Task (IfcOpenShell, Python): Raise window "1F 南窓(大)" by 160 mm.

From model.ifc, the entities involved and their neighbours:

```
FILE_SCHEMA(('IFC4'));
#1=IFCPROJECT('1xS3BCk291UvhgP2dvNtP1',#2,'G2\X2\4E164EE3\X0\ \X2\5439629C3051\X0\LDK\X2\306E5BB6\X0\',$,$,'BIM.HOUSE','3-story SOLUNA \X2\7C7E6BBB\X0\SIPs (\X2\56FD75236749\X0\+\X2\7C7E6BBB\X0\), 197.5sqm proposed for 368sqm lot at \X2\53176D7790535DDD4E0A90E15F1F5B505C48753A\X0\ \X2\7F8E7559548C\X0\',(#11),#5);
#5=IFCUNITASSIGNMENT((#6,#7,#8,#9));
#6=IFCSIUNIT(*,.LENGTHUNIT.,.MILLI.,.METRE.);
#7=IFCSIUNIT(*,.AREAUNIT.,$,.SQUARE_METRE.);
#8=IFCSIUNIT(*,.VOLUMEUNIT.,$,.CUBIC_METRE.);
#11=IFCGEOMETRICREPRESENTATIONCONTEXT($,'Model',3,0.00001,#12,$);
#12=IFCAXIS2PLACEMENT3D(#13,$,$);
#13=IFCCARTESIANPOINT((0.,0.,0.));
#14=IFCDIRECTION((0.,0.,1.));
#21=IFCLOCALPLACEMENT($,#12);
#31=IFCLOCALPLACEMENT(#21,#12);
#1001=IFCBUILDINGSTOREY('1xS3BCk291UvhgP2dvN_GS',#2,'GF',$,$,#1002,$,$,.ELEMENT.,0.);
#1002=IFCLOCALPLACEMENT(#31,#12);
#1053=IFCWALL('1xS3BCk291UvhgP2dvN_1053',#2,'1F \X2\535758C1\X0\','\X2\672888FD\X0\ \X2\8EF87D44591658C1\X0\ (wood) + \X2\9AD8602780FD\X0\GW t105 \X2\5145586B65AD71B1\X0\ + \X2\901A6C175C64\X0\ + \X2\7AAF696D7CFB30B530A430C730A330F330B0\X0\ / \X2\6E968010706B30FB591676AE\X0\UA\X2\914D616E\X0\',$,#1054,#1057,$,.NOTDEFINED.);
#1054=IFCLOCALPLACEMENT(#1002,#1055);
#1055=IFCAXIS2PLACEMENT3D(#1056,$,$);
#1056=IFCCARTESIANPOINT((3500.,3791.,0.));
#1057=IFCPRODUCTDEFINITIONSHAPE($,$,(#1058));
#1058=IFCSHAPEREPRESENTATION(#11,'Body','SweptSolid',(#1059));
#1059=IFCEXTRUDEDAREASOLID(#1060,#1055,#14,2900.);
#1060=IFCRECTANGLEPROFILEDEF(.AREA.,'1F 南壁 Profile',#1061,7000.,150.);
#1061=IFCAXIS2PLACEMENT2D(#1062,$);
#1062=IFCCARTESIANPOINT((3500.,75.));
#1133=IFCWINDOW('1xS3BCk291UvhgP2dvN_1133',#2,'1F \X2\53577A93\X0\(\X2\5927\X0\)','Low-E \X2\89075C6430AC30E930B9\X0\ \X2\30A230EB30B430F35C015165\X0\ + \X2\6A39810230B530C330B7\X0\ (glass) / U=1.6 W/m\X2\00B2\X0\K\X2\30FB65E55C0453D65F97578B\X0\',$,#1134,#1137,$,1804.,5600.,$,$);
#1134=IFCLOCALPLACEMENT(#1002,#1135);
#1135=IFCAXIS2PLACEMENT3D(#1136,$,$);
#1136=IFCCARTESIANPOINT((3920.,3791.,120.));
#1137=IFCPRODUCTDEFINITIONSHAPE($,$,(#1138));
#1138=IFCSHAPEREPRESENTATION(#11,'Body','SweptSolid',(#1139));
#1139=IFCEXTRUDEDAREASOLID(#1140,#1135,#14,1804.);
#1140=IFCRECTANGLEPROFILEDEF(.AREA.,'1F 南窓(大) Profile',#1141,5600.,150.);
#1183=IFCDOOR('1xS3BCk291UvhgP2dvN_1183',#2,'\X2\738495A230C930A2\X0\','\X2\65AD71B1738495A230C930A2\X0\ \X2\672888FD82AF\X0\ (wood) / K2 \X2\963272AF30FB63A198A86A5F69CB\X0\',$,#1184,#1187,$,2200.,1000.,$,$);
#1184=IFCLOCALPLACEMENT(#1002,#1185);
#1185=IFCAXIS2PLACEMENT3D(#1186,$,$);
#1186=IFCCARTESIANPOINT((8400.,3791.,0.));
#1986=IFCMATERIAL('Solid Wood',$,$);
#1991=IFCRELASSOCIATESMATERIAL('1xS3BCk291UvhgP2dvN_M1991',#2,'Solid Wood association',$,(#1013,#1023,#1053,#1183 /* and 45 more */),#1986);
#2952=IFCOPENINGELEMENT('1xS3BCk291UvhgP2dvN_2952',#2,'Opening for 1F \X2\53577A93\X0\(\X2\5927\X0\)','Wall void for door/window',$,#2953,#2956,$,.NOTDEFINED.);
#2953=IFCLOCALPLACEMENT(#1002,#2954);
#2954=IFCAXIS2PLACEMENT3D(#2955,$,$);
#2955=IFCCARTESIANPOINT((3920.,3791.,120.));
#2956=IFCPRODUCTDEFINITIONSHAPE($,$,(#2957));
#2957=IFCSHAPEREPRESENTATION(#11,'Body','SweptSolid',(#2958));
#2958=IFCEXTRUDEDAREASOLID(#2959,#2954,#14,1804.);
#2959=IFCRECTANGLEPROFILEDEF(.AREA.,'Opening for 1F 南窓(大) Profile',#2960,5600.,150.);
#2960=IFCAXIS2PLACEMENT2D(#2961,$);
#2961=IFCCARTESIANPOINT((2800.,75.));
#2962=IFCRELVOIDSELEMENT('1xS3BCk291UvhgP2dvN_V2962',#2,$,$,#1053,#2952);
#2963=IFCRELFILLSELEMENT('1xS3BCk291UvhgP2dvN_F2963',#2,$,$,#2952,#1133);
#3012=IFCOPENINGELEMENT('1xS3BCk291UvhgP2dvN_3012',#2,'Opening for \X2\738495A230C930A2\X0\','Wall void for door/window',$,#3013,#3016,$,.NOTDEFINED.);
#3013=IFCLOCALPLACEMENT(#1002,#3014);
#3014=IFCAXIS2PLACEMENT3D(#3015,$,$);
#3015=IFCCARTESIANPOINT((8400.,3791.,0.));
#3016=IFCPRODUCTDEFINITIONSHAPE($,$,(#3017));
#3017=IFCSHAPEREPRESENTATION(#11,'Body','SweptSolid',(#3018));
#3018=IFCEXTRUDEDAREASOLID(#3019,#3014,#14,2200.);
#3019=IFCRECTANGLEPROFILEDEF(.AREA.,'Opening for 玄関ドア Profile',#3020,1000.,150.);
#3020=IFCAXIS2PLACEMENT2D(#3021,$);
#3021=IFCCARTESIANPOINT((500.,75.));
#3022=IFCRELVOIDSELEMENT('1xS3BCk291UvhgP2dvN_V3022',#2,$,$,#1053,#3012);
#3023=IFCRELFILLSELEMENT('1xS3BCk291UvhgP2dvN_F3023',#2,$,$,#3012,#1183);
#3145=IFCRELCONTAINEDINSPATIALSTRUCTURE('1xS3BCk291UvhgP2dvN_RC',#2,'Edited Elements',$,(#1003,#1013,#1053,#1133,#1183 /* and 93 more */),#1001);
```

```python
import numpy as np
import ifcopenshell
import ifcopenshell.api.geometry
import ifcopenshell.util.placement
import ifcopenshell.util.unit

model = ifcopenshell.open("model.ifc")
unit_scale = ifcopenshell.util.unit.calculate_unit_scale(model)

window = model.by_guid("1xS3BCk291UvhgP2dvN_1133")
opening = window.FillsVoids[0].RelatingOpeningElement
dz = 160.0

shift = np.array([0.0, 0.0, dz])
# The window is not placed relative to its opening, so move both.
for product in (opening, window):
    matrix = ifcopenshell.util.placement.get_local_placement(product.ObjectPlacement)
    matrix[:3, 3] += shift
    ifcopenshell.api.geometry.edit_object_placement(model, product=product, matrix=matrix, is_si=False)

print(f"moved by {dz * unit_scale:+.3f} m")

model.write("model-out.ifc")
```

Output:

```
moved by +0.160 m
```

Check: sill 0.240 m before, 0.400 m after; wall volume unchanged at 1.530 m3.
